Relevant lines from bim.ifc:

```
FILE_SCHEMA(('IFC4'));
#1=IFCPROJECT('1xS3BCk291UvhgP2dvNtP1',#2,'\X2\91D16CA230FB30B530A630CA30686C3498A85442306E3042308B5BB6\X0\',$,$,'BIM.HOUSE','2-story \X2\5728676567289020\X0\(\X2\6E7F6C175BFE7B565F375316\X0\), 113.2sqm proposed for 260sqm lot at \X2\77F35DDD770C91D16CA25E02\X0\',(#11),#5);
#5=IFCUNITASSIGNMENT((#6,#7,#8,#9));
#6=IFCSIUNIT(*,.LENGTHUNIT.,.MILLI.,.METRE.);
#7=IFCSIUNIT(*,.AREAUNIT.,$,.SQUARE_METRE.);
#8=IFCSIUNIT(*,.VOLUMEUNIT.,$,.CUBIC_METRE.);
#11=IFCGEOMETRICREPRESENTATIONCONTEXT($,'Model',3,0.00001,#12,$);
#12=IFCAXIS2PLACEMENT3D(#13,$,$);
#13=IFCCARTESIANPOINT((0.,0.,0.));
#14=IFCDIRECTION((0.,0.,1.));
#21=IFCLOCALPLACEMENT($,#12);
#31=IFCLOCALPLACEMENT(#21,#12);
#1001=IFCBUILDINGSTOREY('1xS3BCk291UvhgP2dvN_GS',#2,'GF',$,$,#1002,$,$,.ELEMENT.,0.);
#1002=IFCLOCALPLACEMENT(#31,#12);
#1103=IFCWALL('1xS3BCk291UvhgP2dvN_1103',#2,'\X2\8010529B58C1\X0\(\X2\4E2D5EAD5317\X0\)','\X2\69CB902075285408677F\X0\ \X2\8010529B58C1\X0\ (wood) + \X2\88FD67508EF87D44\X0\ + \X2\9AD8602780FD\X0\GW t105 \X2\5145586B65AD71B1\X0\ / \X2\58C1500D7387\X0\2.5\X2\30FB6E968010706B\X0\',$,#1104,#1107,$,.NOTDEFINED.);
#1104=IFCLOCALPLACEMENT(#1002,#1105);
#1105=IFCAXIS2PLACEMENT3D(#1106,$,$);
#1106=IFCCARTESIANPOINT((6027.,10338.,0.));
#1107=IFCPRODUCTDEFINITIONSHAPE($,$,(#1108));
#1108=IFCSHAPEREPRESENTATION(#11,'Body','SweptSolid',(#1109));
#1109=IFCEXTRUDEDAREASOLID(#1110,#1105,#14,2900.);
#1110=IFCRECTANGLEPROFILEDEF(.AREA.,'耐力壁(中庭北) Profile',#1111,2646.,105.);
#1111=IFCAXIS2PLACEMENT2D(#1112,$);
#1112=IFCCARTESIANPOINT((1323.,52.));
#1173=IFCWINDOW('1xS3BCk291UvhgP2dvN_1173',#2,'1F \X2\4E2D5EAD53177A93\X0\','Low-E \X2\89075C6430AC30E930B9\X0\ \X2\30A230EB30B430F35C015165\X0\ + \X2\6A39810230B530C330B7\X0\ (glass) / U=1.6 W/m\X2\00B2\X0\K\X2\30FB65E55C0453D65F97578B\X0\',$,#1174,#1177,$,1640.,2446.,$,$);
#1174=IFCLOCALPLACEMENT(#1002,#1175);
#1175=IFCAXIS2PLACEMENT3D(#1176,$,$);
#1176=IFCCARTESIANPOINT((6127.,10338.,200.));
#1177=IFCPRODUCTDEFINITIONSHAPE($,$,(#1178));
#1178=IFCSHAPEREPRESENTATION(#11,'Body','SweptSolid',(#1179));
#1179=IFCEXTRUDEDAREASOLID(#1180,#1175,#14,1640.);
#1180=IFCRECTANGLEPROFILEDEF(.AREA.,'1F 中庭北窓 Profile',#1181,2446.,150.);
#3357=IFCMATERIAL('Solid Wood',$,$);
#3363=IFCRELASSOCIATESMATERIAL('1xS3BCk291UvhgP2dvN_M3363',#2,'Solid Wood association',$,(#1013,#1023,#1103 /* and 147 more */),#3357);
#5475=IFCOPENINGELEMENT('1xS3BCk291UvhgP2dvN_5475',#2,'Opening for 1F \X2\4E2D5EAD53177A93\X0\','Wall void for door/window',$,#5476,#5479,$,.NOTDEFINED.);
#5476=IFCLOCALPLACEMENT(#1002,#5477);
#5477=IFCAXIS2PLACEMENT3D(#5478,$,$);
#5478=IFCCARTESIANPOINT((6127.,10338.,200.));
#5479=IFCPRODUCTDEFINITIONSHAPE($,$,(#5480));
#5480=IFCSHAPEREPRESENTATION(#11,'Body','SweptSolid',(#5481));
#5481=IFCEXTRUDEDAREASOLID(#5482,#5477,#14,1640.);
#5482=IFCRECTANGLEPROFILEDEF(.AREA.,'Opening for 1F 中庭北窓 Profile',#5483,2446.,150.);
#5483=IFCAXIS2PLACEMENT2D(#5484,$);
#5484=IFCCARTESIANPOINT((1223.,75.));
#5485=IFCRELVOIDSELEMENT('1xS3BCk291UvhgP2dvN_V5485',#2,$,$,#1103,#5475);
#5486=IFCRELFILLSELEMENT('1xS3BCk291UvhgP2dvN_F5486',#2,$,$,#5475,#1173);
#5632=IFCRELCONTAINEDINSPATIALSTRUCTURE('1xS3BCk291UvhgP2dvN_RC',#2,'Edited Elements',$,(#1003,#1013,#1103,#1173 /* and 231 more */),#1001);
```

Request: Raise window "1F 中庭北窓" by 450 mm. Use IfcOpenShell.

```python
import numpy as np
import ifcopenshell
import ifcopenshell.api.geometry
import ifcopenshell.util.placement
import ifcopenshell.util.unit

model = ifcopenshell.open("bim.ifc")
unit_scale = ifcopenshell.util.unit.calculate_unit_scale(model)

window = model.by_id(1173)
opening = window.FillsVoids[0].RelatingOpeningElement
dz = 450.0

shift = np.array([0.0, 0.0, dz])
# The window is not placed relative to its opening, so move both.
for product in (opening, window):
    matrix = ifcopenshell.util.placement.get_local_placement(product.ObjectPlacement)
    matrix[:3, 3] += shift
    ifcopenshell.api.geometry.edit_object_placement(model, product=product, matrix=matrix, is_si=False)

print(f"moved by {dz * unit_scale:+.3f} m")

model.write("bim_edited.ifc")
```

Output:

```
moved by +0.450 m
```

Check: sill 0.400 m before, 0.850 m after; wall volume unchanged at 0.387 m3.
